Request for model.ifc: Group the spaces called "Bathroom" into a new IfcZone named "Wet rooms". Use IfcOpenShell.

First a look at what the model holds.

```python
import ifcopenshell

model = ifcopenshell.open("model.ifc")
print(model.schema)
seen = {}
for space in model.by_type("IfcSpace"):
    seen[space.LongName] = seen.get(space.LongName, 0) + 1
for name, count in sorted(seen.items(), key=str):
    print(count, "x", name)
print("zones:", [z.Name for z in model.by_type("IfcZone")][:20])
```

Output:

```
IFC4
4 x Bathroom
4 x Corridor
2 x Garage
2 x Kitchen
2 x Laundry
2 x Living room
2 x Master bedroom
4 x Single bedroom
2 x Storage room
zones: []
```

```python
import ifcopenshell
import ifcopenshell.api.group
import ifcopenshell.api.root

model = ifcopenshell.open("model.ifc")

names = {"Bathroom"}
spaces = [s for s in model.by_type("IfcSpace") if s.LongName in names]

zone = ifcopenshell.api.root.create_entity(model, ifc_class="IfcZone", name="Wet rooms")
ifcopenshell.api.group.assign_group(model, products=spaces, group=zone)
print(len(spaces), "spaces in", zone.Name)

model.write("model_updated.ifc")
```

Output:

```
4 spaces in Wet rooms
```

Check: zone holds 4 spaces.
